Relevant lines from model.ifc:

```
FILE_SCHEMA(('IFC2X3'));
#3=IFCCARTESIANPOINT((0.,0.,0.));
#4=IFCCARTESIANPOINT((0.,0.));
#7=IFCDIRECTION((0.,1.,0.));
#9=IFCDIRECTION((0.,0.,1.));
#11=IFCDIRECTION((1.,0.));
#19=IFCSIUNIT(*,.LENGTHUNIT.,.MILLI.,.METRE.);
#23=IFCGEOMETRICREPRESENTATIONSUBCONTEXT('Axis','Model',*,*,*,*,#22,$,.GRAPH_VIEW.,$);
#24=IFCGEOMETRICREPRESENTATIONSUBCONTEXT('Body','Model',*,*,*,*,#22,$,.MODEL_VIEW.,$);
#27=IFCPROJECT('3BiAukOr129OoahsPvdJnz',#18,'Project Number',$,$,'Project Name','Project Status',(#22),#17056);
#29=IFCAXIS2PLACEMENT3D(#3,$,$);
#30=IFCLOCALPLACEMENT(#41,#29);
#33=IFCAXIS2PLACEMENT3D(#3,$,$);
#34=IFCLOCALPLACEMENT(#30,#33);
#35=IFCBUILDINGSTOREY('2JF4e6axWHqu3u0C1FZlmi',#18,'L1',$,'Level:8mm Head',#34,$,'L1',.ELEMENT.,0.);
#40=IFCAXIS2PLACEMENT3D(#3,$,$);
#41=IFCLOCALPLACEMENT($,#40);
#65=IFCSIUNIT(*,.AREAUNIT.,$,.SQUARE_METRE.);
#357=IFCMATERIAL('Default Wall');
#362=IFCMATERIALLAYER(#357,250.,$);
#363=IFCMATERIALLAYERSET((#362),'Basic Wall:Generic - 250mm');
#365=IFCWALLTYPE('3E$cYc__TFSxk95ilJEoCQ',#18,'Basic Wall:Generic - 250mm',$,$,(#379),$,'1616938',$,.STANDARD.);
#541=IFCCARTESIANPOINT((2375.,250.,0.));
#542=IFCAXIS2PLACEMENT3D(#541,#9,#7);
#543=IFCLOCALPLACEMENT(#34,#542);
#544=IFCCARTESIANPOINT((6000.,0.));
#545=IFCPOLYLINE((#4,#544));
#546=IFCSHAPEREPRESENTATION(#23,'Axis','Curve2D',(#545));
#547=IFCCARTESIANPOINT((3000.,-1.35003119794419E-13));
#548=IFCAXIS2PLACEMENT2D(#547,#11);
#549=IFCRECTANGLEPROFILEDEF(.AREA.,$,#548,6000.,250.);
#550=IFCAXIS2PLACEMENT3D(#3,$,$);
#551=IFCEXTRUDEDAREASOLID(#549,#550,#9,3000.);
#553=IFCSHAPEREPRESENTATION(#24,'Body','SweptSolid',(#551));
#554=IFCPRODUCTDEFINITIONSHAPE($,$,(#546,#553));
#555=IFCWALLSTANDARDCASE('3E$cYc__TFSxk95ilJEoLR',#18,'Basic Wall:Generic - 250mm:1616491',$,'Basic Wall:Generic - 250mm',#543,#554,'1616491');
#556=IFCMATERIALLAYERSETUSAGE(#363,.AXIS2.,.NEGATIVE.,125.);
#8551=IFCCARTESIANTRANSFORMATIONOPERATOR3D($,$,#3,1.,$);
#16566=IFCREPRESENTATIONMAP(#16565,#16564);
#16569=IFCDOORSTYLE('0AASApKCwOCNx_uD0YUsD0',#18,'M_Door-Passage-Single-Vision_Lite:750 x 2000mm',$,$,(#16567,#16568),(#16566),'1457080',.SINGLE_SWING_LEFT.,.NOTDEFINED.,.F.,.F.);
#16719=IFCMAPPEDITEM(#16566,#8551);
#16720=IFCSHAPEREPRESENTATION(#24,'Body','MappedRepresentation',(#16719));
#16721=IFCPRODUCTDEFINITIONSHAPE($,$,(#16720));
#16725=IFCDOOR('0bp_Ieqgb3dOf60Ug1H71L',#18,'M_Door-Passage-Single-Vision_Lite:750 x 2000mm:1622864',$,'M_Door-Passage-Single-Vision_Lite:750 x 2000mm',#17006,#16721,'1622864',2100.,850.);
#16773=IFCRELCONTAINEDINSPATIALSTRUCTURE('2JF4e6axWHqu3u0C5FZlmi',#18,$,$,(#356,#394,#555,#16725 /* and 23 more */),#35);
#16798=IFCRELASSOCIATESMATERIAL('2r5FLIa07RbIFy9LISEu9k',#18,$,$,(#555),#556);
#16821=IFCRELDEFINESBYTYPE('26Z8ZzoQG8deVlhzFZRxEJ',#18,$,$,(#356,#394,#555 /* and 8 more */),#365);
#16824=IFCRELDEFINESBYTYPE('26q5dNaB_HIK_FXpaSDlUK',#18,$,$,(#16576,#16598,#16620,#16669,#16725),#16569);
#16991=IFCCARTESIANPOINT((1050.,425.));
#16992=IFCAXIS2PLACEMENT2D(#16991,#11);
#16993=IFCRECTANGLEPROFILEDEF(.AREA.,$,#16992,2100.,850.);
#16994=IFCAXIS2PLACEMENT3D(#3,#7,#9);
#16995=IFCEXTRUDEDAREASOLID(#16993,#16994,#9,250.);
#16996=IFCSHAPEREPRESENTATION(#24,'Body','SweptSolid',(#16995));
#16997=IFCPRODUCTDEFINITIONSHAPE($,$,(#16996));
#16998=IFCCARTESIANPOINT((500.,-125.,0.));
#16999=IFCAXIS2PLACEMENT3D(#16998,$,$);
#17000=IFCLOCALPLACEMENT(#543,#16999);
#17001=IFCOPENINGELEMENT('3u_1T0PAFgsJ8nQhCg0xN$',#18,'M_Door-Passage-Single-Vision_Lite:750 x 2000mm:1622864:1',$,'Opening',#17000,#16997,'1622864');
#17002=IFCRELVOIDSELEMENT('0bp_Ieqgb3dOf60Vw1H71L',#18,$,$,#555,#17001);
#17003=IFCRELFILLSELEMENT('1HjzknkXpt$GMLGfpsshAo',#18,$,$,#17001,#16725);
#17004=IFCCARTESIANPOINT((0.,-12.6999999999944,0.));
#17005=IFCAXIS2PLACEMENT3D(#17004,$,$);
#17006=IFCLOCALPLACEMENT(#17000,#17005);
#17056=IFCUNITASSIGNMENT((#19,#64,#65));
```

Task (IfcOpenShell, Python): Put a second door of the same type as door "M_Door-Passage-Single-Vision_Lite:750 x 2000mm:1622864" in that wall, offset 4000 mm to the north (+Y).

```python
import ifcopenshell
import ifcopenshell.api.feature
import ifcopenshell.api.geometry
import ifcopenshell.api.root
import ifcopenshell.geom
import ifcopenshell.util.element
import ifcopenshell.util.placement
import ifcopenshell.util.shape

model = ifcopenshell.open("model.ifc")
settings = ifcopenshell.geom.settings()


def volume(element):
    """Net volume in cubic metres, openings subtracted."""
    shape = ifcopenshell.geom.create_shape(settings, element)
    return ifcopenshell.util.shape.get_volume(shape.geometry)


def reuse_history(source, copy):
    """copy_class also copies each property set's owner history, people and application; keep the originals."""
    for rel in copy.IsDefinedBy:
        if rel.is_a("IfcRelDefinesByProperties") and (history := rel.RelatingPropertyDefinition.OwnerHistory):
            rel.RelatingPropertyDefinition.OwnerHistory = source.OwnerHistory
            ifcopenshell.util.element.remove_deep2(model, history)


door = model.by_guid("0bp_Ieqgb3dOf60Ug1H71L")
opening = door.FillsVoids[0].RelatingOpeningElement
wall = opening.VoidsElements[0].RelatingBuildingElement
before = volume(wall)
shift = ifcopenshell.util.placement.get_local_placement(wall.ObjectPlacement)[:3, 0] * 4000.0

# copy_class copies the void relationship, type, container and properties, but no geometry.
new_opening = ifcopenshell.api.root.copy_class(model, product=opening)
new_opening.Representation = ifcopenshell.util.element.copy_deep(
    model, opening.Representation, exclude=["IfcGeometricRepresentationContext", "IfcRepresentationMap"]
)
new_opening.Name = "M_Door-Passage-Single-Vision_Lite:750 x 2000mm"
new_opening.Tag = None
new_door = ifcopenshell.api.root.copy_class(model, product=door)
new_door.Representation = ifcopenshell.util.element.copy_deep(
    model, door.Representation, exclude=["IfcGeometricRepresentationContext", "IfcRepresentationMap"]
)
new_door.Name = "M_Door-Passage-Single-Vision_Lite:750 x 2000mm"
new_door.Tag = None
reuse_history(door, new_door)
fills = ifcopenshell.api.feature.add_filling(model, opening=new_opening, element=new_door)
fills.OwnerHistory = new_door.OwnerHistory  # required in IFC2X3

for old, new in ((opening, new_opening), (door, new_door)):
    matrix = ifcopenshell.util.placement.get_local_placement(old.ObjectPlacement)
    matrix[:3, 3] += shift
    ifcopenshell.api.geometry.edit_object_placement(model, product=new, matrix=matrix, is_si=False)

after = volume(wall)

print(f"wall volume {before:.3f} -> {after:.3f} m3")

model.write("model-out.ifc")
```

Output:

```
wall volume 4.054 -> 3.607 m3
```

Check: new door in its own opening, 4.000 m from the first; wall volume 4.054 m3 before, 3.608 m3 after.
